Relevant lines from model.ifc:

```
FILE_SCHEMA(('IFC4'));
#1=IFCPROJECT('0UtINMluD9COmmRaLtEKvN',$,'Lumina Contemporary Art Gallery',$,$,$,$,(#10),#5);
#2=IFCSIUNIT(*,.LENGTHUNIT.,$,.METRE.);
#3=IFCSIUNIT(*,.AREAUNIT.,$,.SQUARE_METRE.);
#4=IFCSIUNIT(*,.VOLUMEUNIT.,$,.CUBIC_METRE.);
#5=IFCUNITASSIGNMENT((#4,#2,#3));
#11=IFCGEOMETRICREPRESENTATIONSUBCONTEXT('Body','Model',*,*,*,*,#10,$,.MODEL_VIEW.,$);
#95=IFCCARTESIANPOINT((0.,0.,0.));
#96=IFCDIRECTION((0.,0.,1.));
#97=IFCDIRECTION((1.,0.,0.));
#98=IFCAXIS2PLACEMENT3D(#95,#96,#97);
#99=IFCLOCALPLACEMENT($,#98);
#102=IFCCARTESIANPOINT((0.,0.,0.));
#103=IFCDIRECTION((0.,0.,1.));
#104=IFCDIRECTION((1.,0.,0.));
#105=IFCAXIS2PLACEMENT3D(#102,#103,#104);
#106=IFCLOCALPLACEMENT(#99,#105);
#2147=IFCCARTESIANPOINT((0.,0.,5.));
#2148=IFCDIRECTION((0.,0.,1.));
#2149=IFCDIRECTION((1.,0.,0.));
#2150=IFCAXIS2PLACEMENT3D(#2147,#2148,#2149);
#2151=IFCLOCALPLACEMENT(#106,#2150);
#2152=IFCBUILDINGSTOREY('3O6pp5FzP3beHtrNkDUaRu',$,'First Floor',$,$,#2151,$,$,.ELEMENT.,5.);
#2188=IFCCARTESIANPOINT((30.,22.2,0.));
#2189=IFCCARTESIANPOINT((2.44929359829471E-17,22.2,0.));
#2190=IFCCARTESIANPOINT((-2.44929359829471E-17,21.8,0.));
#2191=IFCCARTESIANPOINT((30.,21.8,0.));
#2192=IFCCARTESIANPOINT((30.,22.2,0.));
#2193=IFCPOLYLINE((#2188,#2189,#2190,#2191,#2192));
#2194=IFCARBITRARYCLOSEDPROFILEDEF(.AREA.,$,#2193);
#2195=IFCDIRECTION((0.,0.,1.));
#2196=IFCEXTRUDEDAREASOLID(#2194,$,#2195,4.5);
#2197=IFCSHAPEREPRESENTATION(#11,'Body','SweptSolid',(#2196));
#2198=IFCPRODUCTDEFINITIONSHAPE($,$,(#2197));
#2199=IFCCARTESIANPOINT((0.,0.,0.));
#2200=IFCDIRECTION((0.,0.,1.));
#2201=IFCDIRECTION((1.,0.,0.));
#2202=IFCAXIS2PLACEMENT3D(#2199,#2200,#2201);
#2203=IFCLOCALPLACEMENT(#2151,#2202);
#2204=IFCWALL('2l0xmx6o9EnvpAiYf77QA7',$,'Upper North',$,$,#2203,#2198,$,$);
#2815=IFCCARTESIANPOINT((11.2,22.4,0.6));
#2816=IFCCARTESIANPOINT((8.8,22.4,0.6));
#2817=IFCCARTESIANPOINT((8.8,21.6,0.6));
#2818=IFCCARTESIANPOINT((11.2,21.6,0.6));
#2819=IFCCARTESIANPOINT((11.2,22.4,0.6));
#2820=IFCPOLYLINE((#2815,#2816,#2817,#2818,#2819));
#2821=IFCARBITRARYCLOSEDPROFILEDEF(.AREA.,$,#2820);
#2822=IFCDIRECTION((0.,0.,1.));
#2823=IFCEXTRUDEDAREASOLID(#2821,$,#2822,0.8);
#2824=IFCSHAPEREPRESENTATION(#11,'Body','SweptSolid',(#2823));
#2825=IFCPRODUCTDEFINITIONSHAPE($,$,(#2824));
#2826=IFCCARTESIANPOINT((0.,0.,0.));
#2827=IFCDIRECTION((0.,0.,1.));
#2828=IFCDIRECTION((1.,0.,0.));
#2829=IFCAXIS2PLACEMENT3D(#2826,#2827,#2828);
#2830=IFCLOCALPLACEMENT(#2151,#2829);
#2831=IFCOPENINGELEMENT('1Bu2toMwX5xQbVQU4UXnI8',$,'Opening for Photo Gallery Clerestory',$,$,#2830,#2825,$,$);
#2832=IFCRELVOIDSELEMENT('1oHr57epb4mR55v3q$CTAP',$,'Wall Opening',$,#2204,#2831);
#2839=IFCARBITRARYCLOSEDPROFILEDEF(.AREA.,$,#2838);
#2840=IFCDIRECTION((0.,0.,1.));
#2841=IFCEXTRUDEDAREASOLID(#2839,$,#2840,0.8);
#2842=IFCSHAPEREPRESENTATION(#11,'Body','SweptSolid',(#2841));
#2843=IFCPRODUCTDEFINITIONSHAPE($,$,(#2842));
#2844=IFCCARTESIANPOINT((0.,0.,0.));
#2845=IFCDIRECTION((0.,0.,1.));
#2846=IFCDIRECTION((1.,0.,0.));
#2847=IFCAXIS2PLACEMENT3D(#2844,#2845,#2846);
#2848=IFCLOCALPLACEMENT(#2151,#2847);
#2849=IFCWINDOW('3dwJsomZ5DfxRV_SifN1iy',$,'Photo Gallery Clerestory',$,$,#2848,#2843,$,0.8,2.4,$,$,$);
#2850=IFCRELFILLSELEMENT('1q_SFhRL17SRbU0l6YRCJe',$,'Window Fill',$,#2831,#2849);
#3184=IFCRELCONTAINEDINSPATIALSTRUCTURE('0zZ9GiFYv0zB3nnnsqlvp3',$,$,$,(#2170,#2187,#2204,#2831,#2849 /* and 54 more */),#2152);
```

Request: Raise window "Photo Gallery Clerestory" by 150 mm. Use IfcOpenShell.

```python
import numpy as np
import ifcopenshell
import ifcopenshell.api.geometry
import ifcopenshell.util.placement
import ifcopenshell.util.unit

model = ifcopenshell.open("model.ifc")
unit_scale = ifcopenshell.util.unit.calculate_unit_scale(model)

window = model.by_id(2849)
opening = window.FillsVoids[0].RelatingOpeningElement
dz = 0.15 / unit_scale

shift = np.array([0.0, 0.0, dz])
# The window is not placed relative to its opening, so move both.
for product in (opening, window):
    matrix = ifcopenshell.util.placement.get_local_placement(product.ObjectPlacement)
    matrix[:3, 3] += shift
    ifcopenshell.api.geometry.edit_object_placement(model, product=product, matrix=matrix, is_si=False)

print(f"moved by {dz * unit_scale:+.3f} m")

model.write("model_updated.ifc")
```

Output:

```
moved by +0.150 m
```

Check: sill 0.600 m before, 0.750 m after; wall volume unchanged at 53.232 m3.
